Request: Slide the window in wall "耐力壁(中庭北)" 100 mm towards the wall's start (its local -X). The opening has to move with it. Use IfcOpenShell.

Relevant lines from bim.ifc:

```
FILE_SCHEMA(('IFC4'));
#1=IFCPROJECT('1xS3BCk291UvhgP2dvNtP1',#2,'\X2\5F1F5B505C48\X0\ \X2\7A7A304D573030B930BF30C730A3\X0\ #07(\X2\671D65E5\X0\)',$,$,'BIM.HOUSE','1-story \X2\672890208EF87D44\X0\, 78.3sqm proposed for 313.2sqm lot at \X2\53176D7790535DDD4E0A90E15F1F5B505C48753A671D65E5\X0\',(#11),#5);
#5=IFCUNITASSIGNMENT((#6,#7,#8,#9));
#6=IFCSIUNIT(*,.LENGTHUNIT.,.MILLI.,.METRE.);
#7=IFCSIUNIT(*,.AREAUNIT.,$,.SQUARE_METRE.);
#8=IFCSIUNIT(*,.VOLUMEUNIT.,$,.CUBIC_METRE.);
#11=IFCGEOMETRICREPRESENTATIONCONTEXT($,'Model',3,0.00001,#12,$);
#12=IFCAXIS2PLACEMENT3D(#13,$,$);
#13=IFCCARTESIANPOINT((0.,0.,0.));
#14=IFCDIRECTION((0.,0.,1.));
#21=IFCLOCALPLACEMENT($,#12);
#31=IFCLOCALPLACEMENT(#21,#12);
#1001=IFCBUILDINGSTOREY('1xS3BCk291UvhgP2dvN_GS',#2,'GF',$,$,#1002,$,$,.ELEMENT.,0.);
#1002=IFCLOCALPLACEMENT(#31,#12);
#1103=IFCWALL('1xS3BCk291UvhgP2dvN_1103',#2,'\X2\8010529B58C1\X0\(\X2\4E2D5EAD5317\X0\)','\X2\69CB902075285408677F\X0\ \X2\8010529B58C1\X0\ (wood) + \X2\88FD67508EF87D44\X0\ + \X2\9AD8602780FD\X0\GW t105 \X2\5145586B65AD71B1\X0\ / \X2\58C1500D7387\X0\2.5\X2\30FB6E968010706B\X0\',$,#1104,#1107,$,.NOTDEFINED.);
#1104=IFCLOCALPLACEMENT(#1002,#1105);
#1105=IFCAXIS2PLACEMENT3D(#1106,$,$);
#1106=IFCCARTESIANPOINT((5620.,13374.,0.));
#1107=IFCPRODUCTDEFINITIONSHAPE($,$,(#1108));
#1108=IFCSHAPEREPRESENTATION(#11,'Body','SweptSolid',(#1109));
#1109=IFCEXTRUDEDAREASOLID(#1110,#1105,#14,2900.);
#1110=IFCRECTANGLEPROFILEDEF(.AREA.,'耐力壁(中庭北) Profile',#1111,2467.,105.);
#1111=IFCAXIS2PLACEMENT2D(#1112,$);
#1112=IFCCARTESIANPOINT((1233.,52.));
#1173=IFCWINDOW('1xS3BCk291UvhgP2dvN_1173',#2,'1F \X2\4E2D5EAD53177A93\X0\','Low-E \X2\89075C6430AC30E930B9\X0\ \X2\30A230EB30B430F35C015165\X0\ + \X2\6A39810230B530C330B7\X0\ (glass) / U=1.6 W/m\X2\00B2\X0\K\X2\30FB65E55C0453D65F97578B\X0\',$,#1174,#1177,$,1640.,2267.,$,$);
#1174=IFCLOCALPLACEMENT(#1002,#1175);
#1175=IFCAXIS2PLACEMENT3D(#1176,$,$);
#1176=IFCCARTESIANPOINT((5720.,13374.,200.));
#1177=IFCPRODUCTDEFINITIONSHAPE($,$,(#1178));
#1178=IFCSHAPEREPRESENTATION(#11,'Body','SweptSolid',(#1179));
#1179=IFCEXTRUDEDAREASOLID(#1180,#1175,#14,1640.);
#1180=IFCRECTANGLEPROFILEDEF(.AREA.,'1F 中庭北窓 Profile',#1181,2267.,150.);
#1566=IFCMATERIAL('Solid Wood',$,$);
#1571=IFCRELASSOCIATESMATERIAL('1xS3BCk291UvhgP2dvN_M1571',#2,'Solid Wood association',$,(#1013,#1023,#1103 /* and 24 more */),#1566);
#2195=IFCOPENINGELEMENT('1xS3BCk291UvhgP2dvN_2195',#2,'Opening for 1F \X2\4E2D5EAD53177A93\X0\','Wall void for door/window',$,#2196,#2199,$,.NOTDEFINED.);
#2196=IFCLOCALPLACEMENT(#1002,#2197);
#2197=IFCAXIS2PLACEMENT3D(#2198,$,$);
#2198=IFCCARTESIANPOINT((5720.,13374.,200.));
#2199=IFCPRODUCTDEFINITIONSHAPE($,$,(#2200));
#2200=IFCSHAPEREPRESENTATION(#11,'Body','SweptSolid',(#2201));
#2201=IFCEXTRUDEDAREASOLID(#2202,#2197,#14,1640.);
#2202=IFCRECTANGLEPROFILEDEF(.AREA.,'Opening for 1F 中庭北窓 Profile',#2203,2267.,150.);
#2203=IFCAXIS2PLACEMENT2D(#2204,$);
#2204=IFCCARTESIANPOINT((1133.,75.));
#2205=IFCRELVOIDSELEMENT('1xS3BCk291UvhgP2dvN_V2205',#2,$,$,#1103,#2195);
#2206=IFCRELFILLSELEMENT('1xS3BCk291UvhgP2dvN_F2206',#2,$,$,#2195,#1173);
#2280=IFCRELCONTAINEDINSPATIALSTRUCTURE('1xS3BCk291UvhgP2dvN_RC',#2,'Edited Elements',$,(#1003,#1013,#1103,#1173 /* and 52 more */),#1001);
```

```python
import ifcopenshell
import ifcopenshell.api.geometry
import ifcopenshell.util.placement

model = ifcopenshell.open("bim.ifc")

window = model.by_id(1173)
opening = window.FillsVoids[0].RelatingOpeningElement
wall = opening.VoidsElements[0].RelatingBuildingElement

wall_matrix = ifcopenshell.util.placement.get_local_placement(wall.ObjectPlacement)
shift = wall_matrix[:3, 0] * -100.0
before = ifcopenshell.util.placement.get_local_placement(window.ObjectPlacement)[:3, 3].copy()

# The window is not placed relative to its opening, so move both.
for product in (opening, window):
    matrix = ifcopenshell.util.placement.get_local_placement(product.ObjectPlacement)
    matrix[:3, 3] += shift
    ifcopenshell.api.geometry.edit_object_placement(model, product=product, matrix=matrix, is_si=False)

after = ifcopenshell.util.placement.get_local_placement(window.ObjectPlacement)[:3, 3]
print("window moved by", (after - before).round(3) + 0.0)

model.write("bim_updated.ifc")
```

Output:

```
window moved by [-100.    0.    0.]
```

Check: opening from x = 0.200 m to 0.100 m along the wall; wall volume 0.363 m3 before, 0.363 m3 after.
